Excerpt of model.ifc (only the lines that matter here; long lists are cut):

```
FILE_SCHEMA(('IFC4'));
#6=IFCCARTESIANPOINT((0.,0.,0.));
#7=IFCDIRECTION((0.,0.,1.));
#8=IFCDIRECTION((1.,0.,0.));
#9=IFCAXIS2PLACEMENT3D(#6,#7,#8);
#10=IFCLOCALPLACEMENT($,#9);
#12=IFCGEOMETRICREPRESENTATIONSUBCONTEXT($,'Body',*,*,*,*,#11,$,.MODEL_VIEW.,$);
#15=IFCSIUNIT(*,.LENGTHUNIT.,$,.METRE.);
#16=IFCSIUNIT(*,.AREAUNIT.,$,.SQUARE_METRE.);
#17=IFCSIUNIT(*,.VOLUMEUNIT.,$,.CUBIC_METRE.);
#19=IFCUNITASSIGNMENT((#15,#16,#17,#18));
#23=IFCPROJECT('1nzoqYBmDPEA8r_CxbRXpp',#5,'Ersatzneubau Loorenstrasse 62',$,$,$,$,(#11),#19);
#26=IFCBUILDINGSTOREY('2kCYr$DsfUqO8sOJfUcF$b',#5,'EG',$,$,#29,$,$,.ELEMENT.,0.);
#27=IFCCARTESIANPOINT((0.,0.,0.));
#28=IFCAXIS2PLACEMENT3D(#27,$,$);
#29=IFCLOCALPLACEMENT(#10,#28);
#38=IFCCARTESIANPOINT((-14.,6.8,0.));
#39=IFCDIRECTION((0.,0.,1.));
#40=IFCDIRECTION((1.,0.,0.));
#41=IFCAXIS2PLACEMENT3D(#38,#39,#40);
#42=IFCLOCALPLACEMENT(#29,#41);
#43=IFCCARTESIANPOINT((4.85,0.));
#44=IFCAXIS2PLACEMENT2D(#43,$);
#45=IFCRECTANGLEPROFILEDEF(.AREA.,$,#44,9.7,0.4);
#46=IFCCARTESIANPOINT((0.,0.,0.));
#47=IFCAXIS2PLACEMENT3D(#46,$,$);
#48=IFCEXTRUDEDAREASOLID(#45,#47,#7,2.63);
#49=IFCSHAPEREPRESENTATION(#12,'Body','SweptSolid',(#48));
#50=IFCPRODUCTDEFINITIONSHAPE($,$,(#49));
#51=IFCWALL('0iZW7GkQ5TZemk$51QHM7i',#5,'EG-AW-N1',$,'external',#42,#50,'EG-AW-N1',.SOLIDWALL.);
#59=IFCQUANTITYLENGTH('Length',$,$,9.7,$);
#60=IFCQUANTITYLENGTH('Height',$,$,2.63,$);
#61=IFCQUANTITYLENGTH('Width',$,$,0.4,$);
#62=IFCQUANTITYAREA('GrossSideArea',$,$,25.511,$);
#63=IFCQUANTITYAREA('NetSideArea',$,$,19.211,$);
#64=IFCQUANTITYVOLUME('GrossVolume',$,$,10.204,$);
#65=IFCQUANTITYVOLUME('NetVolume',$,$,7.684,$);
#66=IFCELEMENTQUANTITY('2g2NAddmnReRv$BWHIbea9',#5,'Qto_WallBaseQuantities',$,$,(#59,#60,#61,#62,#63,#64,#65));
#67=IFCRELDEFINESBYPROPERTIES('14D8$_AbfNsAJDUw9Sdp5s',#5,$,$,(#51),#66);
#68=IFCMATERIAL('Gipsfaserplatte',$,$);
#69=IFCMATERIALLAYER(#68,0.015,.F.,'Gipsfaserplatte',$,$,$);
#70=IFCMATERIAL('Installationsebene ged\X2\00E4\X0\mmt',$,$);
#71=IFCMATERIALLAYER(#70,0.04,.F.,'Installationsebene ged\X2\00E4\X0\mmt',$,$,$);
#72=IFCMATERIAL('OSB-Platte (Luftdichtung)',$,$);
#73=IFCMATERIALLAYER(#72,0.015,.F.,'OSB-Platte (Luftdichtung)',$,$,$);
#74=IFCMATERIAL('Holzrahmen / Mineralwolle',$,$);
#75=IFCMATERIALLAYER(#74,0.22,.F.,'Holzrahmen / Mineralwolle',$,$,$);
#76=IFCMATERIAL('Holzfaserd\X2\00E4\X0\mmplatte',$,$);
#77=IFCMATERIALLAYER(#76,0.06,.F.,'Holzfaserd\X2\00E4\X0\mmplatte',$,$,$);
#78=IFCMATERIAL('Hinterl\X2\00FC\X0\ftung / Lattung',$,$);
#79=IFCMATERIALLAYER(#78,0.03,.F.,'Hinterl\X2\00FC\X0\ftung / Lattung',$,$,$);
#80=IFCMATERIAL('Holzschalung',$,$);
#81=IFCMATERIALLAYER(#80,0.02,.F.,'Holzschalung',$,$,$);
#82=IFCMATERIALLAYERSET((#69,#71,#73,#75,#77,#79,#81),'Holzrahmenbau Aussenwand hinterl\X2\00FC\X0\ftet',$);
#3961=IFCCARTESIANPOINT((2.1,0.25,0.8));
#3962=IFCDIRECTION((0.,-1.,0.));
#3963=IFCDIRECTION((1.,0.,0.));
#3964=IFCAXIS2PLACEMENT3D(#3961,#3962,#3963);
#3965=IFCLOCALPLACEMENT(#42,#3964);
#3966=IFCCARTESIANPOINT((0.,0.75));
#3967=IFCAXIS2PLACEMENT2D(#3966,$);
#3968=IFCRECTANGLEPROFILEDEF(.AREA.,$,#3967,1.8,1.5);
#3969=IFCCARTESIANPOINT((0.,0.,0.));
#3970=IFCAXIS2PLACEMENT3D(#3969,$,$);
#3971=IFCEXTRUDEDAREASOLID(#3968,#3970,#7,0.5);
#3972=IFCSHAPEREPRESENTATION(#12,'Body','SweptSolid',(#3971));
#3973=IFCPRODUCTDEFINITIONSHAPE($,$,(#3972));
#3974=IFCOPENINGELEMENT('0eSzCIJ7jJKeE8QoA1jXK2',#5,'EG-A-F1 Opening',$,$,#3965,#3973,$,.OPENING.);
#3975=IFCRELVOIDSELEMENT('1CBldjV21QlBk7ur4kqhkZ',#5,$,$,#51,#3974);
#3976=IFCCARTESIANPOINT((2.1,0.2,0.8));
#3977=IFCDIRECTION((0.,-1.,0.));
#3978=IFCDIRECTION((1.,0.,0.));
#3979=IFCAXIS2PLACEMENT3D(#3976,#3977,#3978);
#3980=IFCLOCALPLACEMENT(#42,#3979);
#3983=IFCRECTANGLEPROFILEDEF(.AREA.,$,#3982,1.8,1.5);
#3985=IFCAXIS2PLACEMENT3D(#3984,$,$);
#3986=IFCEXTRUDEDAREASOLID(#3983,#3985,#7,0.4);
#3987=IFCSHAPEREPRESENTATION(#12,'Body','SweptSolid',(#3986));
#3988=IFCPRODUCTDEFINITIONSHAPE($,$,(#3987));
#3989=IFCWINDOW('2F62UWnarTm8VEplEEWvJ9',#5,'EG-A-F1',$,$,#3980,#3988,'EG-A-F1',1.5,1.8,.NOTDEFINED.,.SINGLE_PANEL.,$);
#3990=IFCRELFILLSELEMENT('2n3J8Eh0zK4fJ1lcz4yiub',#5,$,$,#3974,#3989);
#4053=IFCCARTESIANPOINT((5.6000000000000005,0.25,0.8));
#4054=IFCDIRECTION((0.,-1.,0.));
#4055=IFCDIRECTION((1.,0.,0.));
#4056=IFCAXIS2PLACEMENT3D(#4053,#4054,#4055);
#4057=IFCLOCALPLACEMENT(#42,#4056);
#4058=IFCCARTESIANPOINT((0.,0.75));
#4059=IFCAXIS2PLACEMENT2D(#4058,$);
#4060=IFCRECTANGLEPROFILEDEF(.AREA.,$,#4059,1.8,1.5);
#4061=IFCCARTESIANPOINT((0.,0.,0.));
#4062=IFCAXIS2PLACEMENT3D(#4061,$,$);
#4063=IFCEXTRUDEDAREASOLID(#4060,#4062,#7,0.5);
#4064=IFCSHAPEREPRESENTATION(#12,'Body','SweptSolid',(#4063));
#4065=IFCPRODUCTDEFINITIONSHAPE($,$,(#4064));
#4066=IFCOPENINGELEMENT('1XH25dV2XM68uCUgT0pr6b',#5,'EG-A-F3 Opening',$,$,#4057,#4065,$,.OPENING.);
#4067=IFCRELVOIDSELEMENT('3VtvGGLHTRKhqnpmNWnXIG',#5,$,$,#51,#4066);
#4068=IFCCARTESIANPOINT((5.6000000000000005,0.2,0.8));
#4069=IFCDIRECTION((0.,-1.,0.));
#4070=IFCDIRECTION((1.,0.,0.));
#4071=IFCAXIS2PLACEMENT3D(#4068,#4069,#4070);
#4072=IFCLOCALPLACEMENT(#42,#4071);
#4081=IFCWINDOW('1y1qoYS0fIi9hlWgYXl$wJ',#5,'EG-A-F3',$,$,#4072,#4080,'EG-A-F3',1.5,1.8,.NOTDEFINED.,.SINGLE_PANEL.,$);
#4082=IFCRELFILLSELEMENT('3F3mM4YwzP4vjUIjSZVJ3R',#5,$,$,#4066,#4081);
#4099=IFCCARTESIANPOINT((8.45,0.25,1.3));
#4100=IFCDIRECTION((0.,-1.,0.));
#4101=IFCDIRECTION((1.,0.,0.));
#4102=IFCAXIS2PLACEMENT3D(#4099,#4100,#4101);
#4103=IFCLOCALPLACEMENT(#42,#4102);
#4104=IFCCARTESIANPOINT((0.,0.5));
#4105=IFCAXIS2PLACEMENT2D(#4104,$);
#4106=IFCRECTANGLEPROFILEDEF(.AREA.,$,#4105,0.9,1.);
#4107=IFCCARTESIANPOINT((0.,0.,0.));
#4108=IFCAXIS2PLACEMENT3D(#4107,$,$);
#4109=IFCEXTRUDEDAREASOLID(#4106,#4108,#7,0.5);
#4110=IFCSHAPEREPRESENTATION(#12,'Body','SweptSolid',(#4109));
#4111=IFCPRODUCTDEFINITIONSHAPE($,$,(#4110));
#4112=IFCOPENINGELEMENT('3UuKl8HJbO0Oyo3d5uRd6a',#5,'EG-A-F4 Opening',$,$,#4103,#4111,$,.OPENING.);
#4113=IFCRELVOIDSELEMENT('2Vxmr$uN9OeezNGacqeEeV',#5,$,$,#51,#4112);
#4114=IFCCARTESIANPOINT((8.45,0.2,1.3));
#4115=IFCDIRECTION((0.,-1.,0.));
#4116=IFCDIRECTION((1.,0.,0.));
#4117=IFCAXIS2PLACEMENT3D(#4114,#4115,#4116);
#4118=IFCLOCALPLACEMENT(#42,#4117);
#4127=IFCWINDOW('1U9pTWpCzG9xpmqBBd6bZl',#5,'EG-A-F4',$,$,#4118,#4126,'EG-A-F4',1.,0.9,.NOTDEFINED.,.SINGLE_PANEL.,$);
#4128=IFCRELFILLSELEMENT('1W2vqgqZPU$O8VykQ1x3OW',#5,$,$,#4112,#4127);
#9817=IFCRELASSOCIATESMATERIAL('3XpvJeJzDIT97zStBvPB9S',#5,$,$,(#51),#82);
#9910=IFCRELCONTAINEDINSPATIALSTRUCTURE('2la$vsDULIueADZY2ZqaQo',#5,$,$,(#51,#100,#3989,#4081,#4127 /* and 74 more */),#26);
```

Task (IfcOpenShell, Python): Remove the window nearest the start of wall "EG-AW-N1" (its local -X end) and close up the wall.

```python
import ifcopenshell
import ifcopenshell.api.feature
import ifcopenshell.api.pset
import ifcopenshell.api.root
import ifcopenshell.geom
import ifcopenshell.util.element
import ifcopenshell.util.shape
import ifcopenshell.util.unit

model = ifcopenshell.open("model.ifc")
area_scale = ifcopenshell.util.unit.calculate_unit_scale(model, "AREAUNIT")
volume_scale = ifcopenshell.util.unit.calculate_unit_scale(model, "VOLUMEUNIT")
settings = ifcopenshell.geom.settings()


def volume(element):
    """Net volume in cubic metres, openings subtracted."""
    shape = ifcopenshell.geom.create_shape(settings, element)
    return ifcopenshell.util.shape.get_volume(shape.geometry)


window = model.by_guid("2F62UWnarTm8VEplEEWvJ9")
opening = window.FillsVoids[0].RelatingOpeningElement
wall = opening.VoidsElements[0].RelatingBuildingElement
before = volume(wall)

ifcopenshell.api.root.remove_product(model, product=window)
ifcopenshell.api.feature.remove_feature(model, feature=opening)

after = volume(wall)
thickness = 0.4  # wall thickness in metres

# Update the wall's stored quantities.
qto = model.by_id(ifcopenshell.util.element.get_pset(wall, "Qto_WallBaseQuantities", should_inherit=False)["id"])
ifcopenshell.api.pset.edit_qto(model, qto=qto, properties={
    "NetSideArea": after / thickness / area_scale,
    "NetVolume": after / volume_scale,
})

print(f"wall volume {before:.3f} -> {after:.3f} m3")

model.write("model-out.ifc")
```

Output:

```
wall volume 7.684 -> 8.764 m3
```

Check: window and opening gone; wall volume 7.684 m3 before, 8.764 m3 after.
